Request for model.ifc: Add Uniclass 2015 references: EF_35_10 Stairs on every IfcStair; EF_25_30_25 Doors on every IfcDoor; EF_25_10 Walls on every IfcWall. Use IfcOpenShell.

First a look at what the model holds.

```python
import ifcopenshell

model = ifcopenshell.open("model.ifc")
print(model.schema)
print("classifications:", [c.Name for c in model.by_type("IfcClassification")])
for ifc_class in ("IfcDoor", "IfcRoof", "IfcStair", "IfcWall", "IfcWindow"):
    print(ifc_class, len(model.by_type(ifc_class)))
```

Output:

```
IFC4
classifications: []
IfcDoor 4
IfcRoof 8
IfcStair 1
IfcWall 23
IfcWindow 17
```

```python
import ifcopenshell
import ifcopenshell.api.classification

model = ifcopenshell.open("model.ifc")

system = ifcopenshell.api.classification.add_classification(model, classification="Uniclass 2015")

codes = {
    "IfcStair": ("EF_35_10", "Stairs"),
    "IfcDoor": ("EF_25_30_25", "Doors"),
    "IfcWall": ("EF_25_10", "Walls"),
}
for ifc_class, (code, name) in codes.items():
    products = model.by_type(ifc_class)
    ifcopenshell.api.classification.add_reference(
        model, products=products, classification=system, identification=code, name=name
    )
    print(code, len(products))

model.write("model_edited.ifc")
```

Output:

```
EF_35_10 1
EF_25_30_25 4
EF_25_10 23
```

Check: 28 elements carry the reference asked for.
